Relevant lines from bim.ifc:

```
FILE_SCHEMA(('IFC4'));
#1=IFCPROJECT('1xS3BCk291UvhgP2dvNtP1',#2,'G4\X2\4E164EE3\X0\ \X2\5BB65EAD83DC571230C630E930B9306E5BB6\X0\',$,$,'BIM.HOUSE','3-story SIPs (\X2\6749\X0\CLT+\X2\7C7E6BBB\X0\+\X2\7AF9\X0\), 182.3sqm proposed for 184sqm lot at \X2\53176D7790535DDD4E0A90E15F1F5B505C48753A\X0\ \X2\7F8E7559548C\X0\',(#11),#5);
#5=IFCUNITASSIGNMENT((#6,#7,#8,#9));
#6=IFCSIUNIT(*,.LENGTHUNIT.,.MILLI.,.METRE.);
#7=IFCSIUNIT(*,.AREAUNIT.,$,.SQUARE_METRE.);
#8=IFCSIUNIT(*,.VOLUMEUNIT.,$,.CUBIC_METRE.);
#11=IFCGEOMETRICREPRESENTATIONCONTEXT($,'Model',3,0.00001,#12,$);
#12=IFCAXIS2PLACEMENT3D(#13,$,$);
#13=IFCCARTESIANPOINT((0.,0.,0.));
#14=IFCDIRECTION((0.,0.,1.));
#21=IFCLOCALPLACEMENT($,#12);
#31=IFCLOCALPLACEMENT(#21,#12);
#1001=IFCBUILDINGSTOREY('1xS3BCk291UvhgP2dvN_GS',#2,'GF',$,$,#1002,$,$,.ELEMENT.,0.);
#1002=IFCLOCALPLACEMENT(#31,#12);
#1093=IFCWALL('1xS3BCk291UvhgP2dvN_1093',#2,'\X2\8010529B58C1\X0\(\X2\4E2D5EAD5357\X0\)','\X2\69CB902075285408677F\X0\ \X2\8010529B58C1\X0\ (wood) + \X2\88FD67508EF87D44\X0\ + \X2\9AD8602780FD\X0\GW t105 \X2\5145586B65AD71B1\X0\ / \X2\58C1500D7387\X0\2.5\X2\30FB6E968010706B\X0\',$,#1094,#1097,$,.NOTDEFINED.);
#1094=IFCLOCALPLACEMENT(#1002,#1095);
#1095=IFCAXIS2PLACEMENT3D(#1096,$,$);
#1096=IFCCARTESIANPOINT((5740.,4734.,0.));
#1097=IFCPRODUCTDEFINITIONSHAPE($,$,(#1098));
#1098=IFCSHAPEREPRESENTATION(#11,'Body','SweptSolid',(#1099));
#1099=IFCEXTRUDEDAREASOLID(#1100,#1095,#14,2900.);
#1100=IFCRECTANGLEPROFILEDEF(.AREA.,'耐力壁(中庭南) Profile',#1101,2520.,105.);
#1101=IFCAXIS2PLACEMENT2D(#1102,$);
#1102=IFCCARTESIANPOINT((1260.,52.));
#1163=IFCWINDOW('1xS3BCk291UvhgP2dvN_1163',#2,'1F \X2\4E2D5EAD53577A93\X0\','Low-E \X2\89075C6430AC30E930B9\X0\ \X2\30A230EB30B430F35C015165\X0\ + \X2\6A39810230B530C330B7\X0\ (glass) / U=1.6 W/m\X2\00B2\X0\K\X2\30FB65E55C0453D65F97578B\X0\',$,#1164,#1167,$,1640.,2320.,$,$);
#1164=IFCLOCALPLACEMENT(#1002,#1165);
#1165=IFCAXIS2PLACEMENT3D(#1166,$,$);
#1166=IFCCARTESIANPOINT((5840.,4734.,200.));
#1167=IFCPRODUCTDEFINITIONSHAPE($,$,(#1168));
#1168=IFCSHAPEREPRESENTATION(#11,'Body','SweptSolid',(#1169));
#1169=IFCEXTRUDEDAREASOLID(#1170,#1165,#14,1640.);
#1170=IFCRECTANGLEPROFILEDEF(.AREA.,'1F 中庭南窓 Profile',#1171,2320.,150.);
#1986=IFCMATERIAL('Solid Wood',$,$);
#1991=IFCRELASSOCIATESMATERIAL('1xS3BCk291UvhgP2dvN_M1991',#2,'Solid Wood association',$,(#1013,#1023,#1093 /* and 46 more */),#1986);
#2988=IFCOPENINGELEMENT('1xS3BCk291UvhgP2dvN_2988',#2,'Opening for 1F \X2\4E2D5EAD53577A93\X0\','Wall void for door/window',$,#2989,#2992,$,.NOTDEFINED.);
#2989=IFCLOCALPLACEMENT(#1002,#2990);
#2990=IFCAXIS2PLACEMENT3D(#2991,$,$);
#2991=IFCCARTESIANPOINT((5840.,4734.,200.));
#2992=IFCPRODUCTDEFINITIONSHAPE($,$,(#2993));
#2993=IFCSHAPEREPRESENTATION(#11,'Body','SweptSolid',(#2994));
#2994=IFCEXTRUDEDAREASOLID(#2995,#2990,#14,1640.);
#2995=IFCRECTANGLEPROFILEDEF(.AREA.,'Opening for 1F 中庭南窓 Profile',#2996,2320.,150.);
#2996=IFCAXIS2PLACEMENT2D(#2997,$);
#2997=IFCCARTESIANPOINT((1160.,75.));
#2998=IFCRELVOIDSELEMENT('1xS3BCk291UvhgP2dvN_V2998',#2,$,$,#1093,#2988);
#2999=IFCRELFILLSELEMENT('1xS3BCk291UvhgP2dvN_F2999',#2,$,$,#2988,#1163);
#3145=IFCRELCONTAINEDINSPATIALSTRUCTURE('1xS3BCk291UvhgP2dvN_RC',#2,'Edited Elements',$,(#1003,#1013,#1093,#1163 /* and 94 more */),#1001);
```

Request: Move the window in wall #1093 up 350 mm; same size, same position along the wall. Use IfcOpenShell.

```python
import numpy as np
import ifcopenshell
import ifcopenshell.api.geometry
import ifcopenshell.util.placement
import ifcopenshell.util.unit

model = ifcopenshell.open("bim.ifc")
unit_scale = ifcopenshell.util.unit.calculate_unit_scale(model)

window = model.by_guid("1xS3BCk291UvhgP2dvN_1163")
opening = window.FillsVoids[0].RelatingOpeningElement
dz = 350.0

shift = np.array([0.0, 0.0, dz])
# The window is not placed relative to its opening, so move both.
for product in (opening, window):
    matrix = ifcopenshell.util.placement.get_local_placement(product.ObjectPlacement)
    matrix[:3, 3] += shift
    ifcopenshell.api.geometry.edit_object_placement(model, product=product, matrix=matrix, is_si=False)

print(f"moved by {dz * unit_scale:+.3f} m")

model.write("bim-out.ifc")
```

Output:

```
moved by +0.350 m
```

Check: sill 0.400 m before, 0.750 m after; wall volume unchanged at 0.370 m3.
